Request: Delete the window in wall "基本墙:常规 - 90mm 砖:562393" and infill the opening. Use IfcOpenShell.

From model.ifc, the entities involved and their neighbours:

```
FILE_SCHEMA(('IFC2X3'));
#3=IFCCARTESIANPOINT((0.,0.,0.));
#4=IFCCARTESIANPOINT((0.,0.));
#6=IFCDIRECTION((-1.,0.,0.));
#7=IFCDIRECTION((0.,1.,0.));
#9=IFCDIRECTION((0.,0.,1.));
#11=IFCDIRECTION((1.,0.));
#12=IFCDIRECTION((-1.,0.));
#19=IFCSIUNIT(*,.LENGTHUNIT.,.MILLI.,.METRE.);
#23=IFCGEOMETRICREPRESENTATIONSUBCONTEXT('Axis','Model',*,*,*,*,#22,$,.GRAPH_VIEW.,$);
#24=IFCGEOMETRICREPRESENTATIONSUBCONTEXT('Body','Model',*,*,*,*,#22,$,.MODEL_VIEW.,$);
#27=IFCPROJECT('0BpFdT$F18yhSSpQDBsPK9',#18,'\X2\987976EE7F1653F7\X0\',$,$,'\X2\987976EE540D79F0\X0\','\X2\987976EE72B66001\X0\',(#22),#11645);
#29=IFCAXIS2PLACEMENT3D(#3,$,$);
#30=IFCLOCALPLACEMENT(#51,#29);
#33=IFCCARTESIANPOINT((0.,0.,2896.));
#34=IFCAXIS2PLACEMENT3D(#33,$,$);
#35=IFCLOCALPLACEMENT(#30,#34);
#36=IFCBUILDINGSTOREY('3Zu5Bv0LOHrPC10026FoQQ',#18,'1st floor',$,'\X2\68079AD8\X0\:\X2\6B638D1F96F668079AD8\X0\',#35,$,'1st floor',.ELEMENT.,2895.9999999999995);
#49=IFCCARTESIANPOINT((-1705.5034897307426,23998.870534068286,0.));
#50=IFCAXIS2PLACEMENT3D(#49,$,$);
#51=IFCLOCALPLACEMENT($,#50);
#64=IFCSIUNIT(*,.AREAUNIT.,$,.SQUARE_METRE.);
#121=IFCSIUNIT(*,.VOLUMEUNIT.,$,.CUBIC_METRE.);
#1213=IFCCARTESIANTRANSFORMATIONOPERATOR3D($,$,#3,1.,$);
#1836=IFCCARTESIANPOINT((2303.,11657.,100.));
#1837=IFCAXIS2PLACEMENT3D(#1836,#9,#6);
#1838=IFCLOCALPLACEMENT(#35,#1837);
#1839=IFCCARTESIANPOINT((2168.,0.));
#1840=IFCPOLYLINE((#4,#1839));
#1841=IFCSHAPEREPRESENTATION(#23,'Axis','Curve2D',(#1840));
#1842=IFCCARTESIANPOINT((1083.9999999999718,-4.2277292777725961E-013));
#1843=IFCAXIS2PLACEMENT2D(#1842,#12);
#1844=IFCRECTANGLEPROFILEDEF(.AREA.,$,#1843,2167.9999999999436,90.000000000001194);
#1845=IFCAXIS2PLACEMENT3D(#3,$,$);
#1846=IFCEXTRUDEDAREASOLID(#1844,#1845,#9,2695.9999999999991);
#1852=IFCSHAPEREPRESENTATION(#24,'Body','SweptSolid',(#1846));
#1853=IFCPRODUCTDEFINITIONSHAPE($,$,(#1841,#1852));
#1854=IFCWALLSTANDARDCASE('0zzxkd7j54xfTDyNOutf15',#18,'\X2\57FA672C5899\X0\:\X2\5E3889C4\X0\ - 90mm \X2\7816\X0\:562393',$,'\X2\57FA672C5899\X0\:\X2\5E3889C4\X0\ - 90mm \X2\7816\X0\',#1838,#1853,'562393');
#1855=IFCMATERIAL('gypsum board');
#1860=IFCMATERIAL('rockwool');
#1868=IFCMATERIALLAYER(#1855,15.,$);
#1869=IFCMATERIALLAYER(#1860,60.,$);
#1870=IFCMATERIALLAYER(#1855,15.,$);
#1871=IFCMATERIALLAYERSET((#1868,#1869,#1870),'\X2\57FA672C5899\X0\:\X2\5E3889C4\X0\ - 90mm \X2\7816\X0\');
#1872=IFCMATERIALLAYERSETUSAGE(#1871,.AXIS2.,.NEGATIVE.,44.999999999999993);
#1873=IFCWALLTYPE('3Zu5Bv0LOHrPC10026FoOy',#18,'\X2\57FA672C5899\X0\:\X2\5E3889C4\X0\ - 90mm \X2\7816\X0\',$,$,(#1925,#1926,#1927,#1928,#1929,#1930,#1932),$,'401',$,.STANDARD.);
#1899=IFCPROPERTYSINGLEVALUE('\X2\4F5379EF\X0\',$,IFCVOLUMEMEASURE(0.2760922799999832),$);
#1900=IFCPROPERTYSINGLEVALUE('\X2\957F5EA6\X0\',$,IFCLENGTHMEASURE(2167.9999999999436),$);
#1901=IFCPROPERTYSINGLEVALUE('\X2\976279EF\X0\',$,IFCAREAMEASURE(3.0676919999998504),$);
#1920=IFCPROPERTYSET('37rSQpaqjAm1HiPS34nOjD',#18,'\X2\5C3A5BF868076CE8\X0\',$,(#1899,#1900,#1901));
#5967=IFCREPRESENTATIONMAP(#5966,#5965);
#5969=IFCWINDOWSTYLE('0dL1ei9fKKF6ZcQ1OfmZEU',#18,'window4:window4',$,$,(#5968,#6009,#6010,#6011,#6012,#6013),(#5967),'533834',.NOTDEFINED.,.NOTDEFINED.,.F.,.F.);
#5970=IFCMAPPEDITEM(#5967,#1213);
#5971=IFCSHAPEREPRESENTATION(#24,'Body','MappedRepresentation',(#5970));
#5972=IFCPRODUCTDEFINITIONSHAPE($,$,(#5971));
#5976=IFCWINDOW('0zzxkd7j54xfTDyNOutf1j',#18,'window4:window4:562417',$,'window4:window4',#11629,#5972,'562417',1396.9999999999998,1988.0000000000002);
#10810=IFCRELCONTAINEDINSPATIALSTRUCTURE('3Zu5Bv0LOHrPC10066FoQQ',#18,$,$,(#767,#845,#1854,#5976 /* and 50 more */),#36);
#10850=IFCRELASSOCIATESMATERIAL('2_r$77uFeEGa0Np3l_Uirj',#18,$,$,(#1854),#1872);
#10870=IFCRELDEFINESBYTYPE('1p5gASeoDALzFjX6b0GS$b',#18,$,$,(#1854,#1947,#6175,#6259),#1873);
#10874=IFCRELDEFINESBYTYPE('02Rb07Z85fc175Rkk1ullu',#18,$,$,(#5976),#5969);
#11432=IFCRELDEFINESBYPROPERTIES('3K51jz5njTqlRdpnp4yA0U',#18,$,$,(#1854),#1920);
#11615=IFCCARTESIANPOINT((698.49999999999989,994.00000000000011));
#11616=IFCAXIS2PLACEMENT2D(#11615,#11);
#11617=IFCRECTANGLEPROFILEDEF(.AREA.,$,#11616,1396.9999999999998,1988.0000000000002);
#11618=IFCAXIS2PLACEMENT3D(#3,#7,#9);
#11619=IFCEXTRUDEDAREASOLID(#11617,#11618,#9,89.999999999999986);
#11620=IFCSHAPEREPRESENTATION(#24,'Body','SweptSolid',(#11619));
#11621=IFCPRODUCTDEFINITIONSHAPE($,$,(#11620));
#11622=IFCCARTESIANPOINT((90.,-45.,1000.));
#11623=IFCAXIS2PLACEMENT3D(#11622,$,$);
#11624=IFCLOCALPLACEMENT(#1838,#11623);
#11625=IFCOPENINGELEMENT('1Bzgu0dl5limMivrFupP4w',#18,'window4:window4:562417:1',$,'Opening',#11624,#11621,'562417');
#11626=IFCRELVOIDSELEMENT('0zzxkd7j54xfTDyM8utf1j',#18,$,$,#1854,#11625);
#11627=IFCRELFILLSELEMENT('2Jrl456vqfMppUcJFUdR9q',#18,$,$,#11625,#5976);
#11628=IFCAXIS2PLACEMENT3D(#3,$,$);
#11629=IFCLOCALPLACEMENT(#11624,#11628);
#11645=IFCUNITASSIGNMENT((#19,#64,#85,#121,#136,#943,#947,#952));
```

```python
import ifcopenshell
import ifcopenshell.api.feature
import ifcopenshell.api.pset
import ifcopenshell.api.root
import ifcopenshell.geom
import ifcopenshell.util.element
import ifcopenshell.util.shape
import ifcopenshell.util.unit

model = ifcopenshell.open("model.ifc")
area_scale = ifcopenshell.util.unit.calculate_unit_scale(model, "AREAUNIT")
volume_scale = ifcopenshell.util.unit.calculate_unit_scale(model, "VOLUMEUNIT")
settings = ifcopenshell.geom.settings()


def volume(element):
    """Net volume in cubic metres, openings subtracted."""
    shape = ifcopenshell.geom.create_shape(settings, element)
    return ifcopenshell.util.shape.get_volume(shape.geometry)


window = model.by_guid("0zzxkd7j54xfTDyNOutf1j")
opening = window.FillsVoids[0].RelatingOpeningElement
wall = opening.VoidsElements[0].RelatingBuildingElement
before = volume(wall)

ifcopenshell.api.root.remove_product(model, product=window)
ifcopenshell.api.feature.remove_feature(model, feature=opening)

after = volume(wall)
thickness = 0.09  # wall thickness in metres

# Update the wall's stored quantities.
pset = model.by_id(ifcopenshell.util.element.get_pset(wall, "尺寸标注", should_inherit=False)["id"])
ifcopenshell.api.pset.edit_pset(model, pset=pset, properties={
    "体积": model.create_entity("IfcVolumeMeasure", after / volume_scale),
    "面积": model.create_entity("IfcAreaMeasure", after / thickness / area_scale),
})

print(f"wall volume {before:.3f} -> {after:.3f} m3")

model.write("model-out.ifc")
```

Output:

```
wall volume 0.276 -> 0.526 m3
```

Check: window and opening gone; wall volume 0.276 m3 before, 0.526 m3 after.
